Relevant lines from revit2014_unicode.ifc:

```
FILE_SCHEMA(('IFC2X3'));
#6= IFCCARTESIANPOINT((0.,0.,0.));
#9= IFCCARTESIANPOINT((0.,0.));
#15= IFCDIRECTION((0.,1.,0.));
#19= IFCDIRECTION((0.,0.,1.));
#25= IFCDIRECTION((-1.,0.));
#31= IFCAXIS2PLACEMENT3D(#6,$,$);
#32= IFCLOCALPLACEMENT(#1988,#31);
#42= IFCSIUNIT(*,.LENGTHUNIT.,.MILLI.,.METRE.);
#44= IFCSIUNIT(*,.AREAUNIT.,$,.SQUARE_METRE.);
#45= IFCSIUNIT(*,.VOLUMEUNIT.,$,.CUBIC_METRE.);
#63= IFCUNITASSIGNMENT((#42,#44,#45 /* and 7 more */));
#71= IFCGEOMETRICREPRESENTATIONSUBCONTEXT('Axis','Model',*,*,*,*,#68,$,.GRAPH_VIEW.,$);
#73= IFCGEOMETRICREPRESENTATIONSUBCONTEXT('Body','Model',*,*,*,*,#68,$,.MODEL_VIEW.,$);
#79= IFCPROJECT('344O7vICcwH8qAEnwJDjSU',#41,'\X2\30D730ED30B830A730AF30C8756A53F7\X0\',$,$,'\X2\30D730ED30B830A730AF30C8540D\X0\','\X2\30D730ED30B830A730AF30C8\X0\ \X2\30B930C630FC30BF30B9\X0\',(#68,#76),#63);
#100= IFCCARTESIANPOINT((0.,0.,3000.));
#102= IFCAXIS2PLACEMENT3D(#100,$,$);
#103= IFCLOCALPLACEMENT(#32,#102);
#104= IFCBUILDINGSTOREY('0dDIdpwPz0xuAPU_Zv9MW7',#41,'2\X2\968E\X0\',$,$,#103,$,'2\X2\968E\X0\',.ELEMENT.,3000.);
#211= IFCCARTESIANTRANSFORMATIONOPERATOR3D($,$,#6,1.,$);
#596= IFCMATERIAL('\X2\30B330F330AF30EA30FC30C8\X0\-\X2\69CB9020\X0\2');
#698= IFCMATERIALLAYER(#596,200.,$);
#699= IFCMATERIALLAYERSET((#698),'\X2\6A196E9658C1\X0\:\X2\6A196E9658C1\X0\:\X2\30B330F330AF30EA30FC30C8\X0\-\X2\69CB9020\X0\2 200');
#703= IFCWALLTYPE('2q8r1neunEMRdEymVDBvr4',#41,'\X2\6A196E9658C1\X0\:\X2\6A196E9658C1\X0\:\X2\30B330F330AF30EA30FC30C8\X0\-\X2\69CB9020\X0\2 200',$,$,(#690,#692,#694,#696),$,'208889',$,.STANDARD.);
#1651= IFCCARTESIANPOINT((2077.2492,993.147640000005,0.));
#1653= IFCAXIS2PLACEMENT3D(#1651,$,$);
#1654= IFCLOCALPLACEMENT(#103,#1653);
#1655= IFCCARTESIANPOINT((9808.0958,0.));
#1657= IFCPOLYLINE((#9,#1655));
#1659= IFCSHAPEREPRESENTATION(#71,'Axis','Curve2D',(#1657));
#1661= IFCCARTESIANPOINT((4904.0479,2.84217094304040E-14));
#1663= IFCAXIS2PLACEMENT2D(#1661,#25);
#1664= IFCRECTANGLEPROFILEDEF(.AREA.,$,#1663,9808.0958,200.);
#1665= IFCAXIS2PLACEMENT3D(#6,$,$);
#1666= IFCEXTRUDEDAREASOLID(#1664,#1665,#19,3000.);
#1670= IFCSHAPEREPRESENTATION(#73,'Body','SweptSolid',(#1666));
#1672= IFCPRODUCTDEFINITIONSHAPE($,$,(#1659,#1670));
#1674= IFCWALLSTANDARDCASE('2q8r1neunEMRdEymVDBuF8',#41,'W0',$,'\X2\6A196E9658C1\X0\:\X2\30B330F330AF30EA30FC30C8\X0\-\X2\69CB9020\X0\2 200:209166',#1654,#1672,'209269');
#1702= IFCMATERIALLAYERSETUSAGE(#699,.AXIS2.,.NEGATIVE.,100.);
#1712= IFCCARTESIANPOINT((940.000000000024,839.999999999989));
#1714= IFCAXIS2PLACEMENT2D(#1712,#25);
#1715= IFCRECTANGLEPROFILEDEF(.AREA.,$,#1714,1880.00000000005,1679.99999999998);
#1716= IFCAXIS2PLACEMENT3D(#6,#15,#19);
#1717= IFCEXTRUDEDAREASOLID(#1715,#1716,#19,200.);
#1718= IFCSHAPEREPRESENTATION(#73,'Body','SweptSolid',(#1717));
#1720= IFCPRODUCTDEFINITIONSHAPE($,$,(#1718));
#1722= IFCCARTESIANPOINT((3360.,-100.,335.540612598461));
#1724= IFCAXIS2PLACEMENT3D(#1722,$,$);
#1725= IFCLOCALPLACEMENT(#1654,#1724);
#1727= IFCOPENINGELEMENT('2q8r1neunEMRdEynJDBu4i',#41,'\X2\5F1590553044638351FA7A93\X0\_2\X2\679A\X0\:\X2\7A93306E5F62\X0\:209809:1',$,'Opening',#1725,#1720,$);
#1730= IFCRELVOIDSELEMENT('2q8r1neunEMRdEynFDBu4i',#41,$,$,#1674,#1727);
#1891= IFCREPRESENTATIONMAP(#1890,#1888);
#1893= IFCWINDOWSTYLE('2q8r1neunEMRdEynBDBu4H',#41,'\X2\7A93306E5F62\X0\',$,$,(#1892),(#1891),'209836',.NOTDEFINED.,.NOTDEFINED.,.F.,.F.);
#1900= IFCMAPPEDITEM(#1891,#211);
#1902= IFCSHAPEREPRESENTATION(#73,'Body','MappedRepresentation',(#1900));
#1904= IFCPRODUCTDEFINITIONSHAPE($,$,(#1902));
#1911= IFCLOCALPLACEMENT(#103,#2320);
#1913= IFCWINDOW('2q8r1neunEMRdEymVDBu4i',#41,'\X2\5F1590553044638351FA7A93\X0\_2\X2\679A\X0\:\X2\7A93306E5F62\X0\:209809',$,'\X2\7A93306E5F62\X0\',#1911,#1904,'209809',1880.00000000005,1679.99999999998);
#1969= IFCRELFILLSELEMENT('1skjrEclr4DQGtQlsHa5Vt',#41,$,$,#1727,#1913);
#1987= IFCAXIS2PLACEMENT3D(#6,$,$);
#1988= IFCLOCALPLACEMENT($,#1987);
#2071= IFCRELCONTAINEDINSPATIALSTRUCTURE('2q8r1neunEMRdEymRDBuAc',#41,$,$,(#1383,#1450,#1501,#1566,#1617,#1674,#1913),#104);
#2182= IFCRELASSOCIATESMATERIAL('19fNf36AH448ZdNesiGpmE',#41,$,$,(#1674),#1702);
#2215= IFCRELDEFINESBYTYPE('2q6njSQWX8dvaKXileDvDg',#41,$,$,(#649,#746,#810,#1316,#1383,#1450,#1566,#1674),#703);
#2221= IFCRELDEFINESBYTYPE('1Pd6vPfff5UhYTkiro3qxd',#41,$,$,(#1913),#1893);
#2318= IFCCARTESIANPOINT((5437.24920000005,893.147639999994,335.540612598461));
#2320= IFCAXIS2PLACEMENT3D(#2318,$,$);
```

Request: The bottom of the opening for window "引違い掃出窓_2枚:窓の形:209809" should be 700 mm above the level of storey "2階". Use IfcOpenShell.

```python
import numpy as np
import ifcopenshell
import ifcopenshell.api.geometry
import ifcopenshell.geom
import ifcopenshell.util.element
import ifcopenshell.util.placement
import ifcopenshell.util.shape
import ifcopenshell.util.unit

model = ifcopenshell.open("revit2014_unicode.ifc")
unit_scale = ifcopenshell.util.unit.calculate_unit_scale(model)

window = model.by_guid("2q8r1neunEMRdEymVDBu4i")
opening = window.FillsVoids[0].RelatingOpeningElement
storey = ifcopenshell.util.element.get_container(window, ifc_class="IfcBuildingStorey")
level = ifcopenshell.util.placement.get_local_placement(storey.ObjectPlacement)[2, 3]

# The opening's origin need not be at the sill, so measure its lowest point.
shape = ifcopenshell.geom.create_shape(ifcopenshell.geom.settings(), opening)
bottom = ifcopenshell.util.shape.get_shape_bottom_elevation(shape, shape.geometry) / unit_scale
dz = level + 0.7 / unit_scale - bottom

shift = np.array([0.0, 0.0, dz])
# The window is not placed relative to its opening, so move both.
for product in (opening, window):
    matrix = ifcopenshell.util.placement.get_local_placement(product.ObjectPlacement)
    matrix[:3, 3] += shift
    ifcopenshell.api.geometry.edit_object_placement(model, product=product, matrix=matrix, is_si=False)

print(f"moved by {dz * unit_scale:+.3f} m")

model.write("revit2014_unicode-out.ifc")
```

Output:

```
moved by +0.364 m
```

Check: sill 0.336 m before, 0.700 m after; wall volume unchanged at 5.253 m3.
